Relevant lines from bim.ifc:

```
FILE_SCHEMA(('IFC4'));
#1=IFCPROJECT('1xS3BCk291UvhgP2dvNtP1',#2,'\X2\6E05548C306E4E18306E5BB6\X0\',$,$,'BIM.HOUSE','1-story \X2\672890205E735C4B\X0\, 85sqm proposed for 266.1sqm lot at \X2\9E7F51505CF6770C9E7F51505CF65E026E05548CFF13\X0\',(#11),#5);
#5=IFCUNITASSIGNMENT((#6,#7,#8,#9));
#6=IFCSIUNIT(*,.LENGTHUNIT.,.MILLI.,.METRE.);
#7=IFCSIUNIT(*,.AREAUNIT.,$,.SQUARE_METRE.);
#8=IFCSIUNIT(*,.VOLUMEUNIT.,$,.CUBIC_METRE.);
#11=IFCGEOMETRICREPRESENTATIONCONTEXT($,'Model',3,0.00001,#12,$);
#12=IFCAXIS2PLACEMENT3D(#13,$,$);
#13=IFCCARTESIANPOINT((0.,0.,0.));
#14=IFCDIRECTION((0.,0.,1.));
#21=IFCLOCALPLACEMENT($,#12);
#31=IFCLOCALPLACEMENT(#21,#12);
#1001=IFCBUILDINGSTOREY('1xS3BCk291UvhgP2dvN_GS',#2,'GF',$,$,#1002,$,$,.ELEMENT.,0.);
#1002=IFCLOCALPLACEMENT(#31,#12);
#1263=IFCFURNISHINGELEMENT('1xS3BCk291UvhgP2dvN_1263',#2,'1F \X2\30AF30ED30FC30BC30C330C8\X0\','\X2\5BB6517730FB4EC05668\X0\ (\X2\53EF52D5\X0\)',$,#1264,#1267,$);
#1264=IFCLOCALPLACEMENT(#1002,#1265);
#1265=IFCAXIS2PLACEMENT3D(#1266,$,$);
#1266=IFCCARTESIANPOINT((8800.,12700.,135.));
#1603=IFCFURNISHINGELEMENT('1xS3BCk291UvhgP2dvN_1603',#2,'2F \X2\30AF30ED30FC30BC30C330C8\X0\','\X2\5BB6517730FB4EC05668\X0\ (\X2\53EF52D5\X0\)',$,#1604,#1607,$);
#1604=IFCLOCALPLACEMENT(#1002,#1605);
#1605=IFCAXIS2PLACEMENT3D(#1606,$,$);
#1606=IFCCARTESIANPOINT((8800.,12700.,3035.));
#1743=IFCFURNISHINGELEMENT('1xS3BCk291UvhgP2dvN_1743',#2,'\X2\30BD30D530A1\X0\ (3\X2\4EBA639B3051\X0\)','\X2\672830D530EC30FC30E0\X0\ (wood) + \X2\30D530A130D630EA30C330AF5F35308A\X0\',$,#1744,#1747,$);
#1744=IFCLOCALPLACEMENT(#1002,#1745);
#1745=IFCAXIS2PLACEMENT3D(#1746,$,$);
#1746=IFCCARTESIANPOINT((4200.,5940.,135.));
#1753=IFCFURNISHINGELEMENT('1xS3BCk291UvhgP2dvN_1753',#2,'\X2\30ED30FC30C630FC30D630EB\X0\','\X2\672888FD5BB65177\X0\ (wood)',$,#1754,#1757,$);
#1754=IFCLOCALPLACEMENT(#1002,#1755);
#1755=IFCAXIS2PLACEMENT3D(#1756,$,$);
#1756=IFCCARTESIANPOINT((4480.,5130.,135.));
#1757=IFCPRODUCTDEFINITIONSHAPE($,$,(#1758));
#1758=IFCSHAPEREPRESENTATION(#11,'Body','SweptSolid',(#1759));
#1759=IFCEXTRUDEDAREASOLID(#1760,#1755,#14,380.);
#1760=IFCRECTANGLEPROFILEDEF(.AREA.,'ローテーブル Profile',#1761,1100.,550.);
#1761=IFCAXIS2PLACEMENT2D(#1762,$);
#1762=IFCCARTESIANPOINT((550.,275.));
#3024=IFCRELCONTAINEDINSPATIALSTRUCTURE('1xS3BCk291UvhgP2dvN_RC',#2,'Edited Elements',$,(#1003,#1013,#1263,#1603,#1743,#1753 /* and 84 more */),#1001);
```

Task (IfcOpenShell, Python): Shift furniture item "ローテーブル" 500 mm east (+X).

```python
import ifcopenshell
import ifcopenshell.api.geometry
import ifcopenshell.util.placement

model = ifcopenshell.open("bim.ifc")

item = model.by_guid("1xS3BCk291UvhgP2dvN_1753")
matrix = ifcopenshell.util.placement.get_local_placement(item.ObjectPlacement)
matrix[0, 3] += 500.0
ifcopenshell.api.geometry.edit_object_placement(model, product=item, matrix=matrix, is_si=False)

print(ifcopenshell.util.placement.get_local_placement(item.ObjectPlacement).round(3) + 0.0)

model.write("bim_edited.ifc")
```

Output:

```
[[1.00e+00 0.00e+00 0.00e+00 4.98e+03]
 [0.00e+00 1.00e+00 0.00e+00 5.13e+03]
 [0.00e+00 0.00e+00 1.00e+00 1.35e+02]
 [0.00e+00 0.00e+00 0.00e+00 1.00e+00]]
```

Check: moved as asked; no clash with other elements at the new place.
